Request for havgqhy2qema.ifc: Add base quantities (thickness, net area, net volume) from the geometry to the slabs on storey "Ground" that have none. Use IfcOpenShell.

First a look at what the model holds.

```python
import ifcopenshell
import ifcopenshell.util.element
import ifcopenshell.util.unit

model = ifcopenshell.open("havgqhy2qema.ifc")
print(model.schema)
for unit_type in ("LENGTHUNIT", "AREAUNIT", "VOLUMEUNIT"):
    print(unit_type, ifcopenshell.util.unit.calculate_unit_scale(model, unit_type))
storey = next(s for s in model.by_type("IfcBuildingStorey") if s.Name == "Ground")
slabs = [e for e in ifcopenshell.util.element.get_decomposition(storey) if e.is_a("IfcSlab")]
for e in sorted(slabs, key=lambda e: e.id()):
    print(e.id(), e.is_a(), e.Name, list(ifcopenshell.util.element.get_psets(e, qtos_only=True)), sep=" | ")
```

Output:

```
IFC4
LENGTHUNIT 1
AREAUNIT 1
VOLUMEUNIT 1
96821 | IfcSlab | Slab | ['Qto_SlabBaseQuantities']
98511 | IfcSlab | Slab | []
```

```python
import ifcopenshell
import ifcopenshell.api.pset
import ifcopenshell.geom
import ifcopenshell.util.element
import ifcopenshell.util.shape
import ifcopenshell.util.unit

model = ifcopenshell.open("havgqhy2qema.ifc")
unit_scale = ifcopenshell.util.unit.calculate_unit_scale(model)
area_scale = ifcopenshell.util.unit.calculate_unit_scale(model, "AREAUNIT")
volume_scale = ifcopenshell.util.unit.calculate_unit_scale(model, "VOLUMEUNIT")
settings = ifcopenshell.geom.settings()

storey = next(s for s in model.by_type("IfcBuildingStorey") if s.Name == "Ground")
slabs = [e for e in ifcopenshell.util.element.get_decomposition(storey) if e.is_a("IfcSlab")]

for e in sorted(slabs, key=lambda e: e.id()):
    if ifcopenshell.util.element.get_psets(e, qtos_only=True, should_inherit=False):
        continue
    # Geometry comes back in metres, in the element's own axes.
    shape = ifcopenshell.geom.create_shape(settings, e)
    values = {
        "Width": ifcopenshell.util.shape.get_z(shape.geometry) / unit_scale,
        "NetArea": ifcopenshell.util.shape.get_footprint_area(shape.geometry) / area_scale,
        "NetVolume": ifcopenshell.util.shape.get_volume(shape.geometry) / volume_scale,
    }
    qto = ifcopenshell.api.pset.add_qto(model, product=e, name="Qto_SlabBaseQuantities")
    ifcopenshell.api.pset.edit_qto(model, qto=qto, properties=values)
    print(e.id(), {k: round(v, 3) for k, v in values.items()})

model.write("havgqhy2qema-out.ifc")
```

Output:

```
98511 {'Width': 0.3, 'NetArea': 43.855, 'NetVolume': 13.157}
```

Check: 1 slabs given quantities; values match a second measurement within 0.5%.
